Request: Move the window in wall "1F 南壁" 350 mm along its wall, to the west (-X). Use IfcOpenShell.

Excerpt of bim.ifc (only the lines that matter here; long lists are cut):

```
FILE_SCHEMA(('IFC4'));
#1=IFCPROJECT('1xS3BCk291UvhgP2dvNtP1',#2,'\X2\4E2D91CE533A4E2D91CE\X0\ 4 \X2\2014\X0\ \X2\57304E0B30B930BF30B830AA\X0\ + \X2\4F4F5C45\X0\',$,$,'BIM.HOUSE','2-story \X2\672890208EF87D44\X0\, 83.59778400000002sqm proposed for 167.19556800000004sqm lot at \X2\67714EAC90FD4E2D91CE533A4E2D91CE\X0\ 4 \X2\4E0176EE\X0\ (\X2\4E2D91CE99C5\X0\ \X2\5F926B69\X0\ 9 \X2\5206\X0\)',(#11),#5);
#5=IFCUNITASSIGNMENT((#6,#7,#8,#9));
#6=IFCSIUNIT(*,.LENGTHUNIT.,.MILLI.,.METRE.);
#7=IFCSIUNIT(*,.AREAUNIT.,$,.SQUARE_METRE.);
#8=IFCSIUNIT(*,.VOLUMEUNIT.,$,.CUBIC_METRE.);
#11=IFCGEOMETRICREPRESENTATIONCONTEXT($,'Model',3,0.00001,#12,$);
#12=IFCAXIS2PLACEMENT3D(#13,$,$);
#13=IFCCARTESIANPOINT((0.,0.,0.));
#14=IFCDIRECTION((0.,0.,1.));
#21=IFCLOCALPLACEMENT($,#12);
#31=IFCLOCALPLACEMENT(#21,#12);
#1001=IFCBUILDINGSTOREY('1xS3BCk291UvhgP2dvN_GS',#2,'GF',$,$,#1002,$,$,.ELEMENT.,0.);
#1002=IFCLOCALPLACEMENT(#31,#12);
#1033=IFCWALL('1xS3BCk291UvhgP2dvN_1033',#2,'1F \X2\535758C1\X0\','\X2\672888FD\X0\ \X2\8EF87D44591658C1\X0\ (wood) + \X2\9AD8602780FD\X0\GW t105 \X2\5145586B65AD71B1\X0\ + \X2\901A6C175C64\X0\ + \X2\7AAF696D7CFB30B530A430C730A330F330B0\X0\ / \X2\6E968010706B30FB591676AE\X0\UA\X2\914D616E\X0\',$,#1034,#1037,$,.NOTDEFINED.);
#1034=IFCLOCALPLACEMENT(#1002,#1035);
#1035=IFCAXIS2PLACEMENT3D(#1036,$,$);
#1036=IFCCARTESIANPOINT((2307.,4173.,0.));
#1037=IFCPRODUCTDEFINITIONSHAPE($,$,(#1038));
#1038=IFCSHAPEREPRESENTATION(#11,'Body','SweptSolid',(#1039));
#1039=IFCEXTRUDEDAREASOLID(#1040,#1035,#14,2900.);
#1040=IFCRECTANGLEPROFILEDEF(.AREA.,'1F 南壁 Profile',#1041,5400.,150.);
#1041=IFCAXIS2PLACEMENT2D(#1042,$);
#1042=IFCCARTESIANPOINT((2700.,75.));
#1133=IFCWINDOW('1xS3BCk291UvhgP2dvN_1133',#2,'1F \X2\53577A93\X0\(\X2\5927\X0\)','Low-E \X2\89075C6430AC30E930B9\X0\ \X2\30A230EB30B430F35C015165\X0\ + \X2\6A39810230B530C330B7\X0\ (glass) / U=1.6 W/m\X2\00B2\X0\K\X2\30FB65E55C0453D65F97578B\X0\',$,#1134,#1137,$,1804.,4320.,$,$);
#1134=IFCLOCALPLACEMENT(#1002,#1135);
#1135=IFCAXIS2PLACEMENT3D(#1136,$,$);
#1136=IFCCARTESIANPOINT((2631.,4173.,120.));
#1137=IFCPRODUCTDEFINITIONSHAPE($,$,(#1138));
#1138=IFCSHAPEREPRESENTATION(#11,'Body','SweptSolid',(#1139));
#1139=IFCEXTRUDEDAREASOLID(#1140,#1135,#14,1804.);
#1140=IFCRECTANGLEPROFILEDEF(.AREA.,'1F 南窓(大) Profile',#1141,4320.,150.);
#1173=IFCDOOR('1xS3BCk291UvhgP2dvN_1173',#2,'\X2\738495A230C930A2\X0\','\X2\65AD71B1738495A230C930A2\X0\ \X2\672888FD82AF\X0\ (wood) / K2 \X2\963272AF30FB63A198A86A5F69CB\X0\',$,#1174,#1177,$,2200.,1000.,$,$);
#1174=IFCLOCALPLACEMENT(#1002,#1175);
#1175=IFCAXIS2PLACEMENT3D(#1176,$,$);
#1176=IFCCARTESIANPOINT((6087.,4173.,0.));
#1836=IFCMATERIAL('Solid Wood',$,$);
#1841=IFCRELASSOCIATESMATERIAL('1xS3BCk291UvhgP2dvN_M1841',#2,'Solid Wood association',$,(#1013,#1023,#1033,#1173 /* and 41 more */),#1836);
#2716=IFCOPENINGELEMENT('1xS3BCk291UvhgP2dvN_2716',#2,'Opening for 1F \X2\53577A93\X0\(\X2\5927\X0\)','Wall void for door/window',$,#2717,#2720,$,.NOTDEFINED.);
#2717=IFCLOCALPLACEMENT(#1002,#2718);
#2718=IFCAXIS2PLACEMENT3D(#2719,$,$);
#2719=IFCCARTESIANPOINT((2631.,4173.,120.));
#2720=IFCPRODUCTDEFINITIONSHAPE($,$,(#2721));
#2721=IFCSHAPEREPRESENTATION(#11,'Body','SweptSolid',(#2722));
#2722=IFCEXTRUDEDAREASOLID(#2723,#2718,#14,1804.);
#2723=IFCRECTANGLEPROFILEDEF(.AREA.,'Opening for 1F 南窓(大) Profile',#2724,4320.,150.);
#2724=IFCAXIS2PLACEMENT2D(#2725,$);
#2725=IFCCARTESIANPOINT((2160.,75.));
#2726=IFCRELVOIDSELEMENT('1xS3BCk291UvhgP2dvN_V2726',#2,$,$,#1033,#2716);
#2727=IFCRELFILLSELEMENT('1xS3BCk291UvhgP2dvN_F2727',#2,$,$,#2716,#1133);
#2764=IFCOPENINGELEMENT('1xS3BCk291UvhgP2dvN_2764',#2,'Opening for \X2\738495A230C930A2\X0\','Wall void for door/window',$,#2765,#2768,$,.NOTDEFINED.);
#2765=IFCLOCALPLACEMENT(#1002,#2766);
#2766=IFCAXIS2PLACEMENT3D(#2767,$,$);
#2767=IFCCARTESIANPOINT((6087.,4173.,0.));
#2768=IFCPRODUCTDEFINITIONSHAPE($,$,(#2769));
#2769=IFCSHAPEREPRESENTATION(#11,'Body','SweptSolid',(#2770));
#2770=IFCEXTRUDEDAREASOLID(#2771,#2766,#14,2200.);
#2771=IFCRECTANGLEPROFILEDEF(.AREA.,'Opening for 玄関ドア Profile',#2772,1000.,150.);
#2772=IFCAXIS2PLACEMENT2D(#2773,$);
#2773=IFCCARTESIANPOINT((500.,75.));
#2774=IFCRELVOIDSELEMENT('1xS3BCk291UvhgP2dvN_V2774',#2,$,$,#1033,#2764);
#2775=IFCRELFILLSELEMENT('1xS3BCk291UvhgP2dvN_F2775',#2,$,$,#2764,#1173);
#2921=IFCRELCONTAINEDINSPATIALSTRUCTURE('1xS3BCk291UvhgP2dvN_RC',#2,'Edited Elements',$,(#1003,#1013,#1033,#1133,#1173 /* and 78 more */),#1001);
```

```python
import ifcopenshell
import ifcopenshell.api.geometry
import ifcopenshell.util.placement

model = ifcopenshell.open("bim.ifc")

window = model.by_guid("1xS3BCk291UvhgP2dvN_1133")
opening = window.FillsVoids[0].RelatingOpeningElement
wall = opening.VoidsElements[0].RelatingBuildingElement

wall_matrix = ifcopenshell.util.placement.get_local_placement(wall.ObjectPlacement)
shift = wall_matrix[:3, 0] * -350.0
before = ifcopenshell.util.placement.get_local_placement(window.ObjectPlacement)[:3, 3].copy()

# The window is not placed relative to its opening, so move both.
for product in (opening, window):
    matrix = ifcopenshell.util.placement.get_local_placement(product.ObjectPlacement)
    matrix[:3, 3] += shift
    ifcopenshell.api.geometry.edit_object_placement(model, product=product, matrix=matrix, is_si=False)

after = ifcopenshell.util.placement.get_local_placement(window.ObjectPlacement)[:3, 3]
print("window moved by", (after - before).round(3) + 0.0)

model.write("bim_updated.ifc")
```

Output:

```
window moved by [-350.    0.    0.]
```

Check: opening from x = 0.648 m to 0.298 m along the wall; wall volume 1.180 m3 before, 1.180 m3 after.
